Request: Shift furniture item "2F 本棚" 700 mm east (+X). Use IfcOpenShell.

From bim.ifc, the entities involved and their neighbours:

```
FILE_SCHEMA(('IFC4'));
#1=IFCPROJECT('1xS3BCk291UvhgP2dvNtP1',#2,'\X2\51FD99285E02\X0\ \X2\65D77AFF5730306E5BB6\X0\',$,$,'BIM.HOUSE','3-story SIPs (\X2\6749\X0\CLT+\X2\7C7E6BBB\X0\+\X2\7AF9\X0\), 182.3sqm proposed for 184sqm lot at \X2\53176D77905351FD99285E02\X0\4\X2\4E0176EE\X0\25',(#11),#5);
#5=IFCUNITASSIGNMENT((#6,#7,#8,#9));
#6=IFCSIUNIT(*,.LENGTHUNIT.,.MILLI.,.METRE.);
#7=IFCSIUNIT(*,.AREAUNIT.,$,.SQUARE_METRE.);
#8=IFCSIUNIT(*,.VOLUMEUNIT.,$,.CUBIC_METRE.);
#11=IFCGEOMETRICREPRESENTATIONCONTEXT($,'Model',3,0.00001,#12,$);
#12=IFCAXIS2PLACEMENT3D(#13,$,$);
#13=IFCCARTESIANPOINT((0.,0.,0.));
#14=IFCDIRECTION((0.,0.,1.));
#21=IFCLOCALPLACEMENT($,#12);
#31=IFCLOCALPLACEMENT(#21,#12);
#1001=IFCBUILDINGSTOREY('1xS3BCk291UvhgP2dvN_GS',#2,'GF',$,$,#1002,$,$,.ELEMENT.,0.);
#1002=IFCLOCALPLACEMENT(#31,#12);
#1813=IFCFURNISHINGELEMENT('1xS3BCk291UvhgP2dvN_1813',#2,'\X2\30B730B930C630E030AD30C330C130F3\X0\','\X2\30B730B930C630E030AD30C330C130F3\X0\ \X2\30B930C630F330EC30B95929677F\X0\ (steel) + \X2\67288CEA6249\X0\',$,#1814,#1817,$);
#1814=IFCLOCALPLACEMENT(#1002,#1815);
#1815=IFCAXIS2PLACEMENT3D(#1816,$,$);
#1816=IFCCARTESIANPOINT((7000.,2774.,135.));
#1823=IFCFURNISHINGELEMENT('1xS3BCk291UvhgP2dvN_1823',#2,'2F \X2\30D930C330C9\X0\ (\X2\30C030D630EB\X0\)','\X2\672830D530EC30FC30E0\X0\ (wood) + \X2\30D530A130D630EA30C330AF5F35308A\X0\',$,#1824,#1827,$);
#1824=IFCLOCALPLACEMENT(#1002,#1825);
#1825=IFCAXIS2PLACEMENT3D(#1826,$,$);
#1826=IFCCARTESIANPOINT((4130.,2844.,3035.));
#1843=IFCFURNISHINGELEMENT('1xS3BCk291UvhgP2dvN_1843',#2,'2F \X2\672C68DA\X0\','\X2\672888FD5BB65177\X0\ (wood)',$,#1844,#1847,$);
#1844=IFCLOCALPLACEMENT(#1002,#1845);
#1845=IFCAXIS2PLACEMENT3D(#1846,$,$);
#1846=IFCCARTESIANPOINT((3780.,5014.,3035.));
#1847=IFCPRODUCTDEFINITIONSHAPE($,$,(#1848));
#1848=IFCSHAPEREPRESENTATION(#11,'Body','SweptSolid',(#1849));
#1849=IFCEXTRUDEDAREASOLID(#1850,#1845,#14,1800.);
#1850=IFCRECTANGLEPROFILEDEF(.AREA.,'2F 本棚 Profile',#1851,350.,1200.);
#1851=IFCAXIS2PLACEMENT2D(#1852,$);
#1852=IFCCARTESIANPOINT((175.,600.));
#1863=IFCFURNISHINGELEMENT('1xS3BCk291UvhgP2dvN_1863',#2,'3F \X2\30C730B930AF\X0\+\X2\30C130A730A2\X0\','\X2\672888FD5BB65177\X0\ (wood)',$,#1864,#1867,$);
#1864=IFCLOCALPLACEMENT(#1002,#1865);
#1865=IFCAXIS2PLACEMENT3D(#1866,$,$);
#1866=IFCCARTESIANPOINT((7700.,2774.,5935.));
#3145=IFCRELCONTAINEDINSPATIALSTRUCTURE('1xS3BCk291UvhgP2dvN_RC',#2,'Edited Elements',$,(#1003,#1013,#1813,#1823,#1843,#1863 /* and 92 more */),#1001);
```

```python
import ifcopenshell
import ifcopenshell.api.geometry
import ifcopenshell.util.placement
import ifcopenshell.util.unit

model = ifcopenshell.open("bim.ifc")
unit_scale = ifcopenshell.util.unit.calculate_unit_scale(model)

item = model.by_id(1843)
matrix = ifcopenshell.util.placement.get_local_placement(item.ObjectPlacement)
matrix[0, 3] += 0.7 / unit_scale
ifcopenshell.api.geometry.edit_object_placement(model, product=item, matrix=matrix, is_si=False)

print(ifcopenshell.util.placement.get_local_placement(item.ObjectPlacement).round(3) + 0.0)

model.write("bim_rev.ifc")
```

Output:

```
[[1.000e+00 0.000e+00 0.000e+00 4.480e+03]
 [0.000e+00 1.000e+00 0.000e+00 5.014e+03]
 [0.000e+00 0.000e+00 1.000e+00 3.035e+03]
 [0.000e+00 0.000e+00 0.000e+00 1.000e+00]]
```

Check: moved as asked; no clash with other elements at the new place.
